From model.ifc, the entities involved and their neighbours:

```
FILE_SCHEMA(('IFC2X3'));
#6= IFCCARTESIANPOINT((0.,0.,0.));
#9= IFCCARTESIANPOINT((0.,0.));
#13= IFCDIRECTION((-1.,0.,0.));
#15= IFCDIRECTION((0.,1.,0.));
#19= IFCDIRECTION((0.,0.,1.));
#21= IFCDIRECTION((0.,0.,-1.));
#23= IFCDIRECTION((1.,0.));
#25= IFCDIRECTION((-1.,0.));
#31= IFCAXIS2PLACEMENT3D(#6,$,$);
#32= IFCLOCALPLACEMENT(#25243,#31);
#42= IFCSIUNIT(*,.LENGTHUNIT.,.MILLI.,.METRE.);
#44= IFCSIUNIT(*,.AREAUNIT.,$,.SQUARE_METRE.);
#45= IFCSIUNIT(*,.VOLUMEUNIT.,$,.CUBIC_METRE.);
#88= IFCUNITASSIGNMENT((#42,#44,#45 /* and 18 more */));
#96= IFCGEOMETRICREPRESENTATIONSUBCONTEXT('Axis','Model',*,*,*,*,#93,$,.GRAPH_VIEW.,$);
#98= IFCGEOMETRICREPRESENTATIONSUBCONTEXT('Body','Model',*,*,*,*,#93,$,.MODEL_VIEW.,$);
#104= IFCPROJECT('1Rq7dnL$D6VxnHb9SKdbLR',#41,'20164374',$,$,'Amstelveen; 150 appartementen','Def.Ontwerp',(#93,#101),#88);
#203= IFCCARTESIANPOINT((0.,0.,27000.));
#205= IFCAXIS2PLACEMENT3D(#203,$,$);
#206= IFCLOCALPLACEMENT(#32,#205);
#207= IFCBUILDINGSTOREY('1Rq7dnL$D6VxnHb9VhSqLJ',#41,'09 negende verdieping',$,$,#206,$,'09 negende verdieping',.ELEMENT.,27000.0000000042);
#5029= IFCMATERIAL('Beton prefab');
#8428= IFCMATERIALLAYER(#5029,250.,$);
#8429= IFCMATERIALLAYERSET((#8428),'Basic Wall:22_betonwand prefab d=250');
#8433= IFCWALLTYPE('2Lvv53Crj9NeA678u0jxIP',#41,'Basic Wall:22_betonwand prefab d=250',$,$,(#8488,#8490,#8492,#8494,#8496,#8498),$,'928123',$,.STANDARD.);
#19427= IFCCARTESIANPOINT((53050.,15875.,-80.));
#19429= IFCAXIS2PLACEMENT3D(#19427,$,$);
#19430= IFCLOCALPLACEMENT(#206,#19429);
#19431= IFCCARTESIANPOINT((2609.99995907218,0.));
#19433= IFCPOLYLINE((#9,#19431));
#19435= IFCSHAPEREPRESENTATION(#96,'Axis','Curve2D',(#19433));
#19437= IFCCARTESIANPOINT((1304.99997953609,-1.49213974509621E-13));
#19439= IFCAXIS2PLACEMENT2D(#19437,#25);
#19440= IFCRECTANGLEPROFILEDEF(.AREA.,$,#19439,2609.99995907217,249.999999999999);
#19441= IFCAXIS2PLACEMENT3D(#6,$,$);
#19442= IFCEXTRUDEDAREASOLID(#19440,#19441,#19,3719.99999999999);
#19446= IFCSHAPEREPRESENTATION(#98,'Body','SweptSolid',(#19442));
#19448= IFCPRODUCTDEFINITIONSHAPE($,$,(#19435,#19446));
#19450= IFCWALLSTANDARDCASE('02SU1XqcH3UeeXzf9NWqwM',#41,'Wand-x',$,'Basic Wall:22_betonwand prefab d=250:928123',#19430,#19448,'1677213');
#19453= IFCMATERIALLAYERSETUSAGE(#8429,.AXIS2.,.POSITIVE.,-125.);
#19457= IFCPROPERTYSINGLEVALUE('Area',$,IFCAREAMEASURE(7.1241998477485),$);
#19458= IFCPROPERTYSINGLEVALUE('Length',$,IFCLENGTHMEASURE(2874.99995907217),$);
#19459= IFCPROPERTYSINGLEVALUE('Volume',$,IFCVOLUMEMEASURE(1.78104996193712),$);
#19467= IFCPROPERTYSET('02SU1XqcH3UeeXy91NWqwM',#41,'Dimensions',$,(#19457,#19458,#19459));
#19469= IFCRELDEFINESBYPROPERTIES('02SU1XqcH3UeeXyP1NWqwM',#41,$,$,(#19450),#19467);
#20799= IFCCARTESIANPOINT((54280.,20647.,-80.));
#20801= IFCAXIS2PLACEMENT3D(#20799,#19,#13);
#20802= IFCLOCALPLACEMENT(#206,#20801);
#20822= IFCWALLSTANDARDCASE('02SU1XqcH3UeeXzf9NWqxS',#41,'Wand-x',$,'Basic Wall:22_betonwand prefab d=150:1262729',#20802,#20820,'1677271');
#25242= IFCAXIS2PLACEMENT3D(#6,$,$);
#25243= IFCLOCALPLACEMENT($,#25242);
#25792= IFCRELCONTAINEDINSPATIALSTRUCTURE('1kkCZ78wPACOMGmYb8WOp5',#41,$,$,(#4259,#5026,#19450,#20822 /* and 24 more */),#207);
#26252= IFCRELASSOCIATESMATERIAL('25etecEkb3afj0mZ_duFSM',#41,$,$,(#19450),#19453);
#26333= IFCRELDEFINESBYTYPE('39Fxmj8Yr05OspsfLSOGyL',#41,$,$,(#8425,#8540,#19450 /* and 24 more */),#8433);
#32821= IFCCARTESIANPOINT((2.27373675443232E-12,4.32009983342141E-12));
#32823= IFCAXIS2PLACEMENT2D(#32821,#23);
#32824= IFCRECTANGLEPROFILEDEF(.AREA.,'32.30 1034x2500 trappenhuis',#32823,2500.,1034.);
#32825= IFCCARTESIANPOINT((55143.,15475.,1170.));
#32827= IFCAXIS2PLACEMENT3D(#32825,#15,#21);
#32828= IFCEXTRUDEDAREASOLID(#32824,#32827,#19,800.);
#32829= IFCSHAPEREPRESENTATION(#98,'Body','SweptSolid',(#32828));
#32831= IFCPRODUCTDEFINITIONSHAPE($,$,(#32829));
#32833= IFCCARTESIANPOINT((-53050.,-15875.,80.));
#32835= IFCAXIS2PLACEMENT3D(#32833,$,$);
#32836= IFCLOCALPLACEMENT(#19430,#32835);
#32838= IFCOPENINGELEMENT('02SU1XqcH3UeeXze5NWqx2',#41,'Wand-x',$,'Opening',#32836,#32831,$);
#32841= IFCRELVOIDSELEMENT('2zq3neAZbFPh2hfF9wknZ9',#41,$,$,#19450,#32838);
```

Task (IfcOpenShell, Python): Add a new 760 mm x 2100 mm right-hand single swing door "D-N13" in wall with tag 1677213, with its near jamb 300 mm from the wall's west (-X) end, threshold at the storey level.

```python
import numpy as np
import ifcopenshell
import ifcopenshell.api.feature
import ifcopenshell.api.geometry
import ifcopenshell.api.pset
import ifcopenshell.api.root
import ifcopenshell.api.spatial
import ifcopenshell.api.type
import ifcopenshell.geom
import ifcopenshell.util.element
import ifcopenshell.util.placement
import ifcopenshell.util.representation
import ifcopenshell.util.shape
import ifcopenshell.util.unit

model = ifcopenshell.open("model.ifc")
unit_scale = ifcopenshell.util.unit.calculate_unit_scale(model)
area_scale = ifcopenshell.util.unit.calculate_unit_scale(model, "AREAUNIT")
volume_scale = ifcopenshell.util.unit.calculate_unit_scale(model, "VOLUMEUNIT")
settings = ifcopenshell.geom.settings()


def volume(element):
    """Net volume in cubic metres, openings subtracted."""
    shape = ifcopenshell.geom.create_shape(settings, element)
    return ifcopenshell.util.shape.get_volume(shape.geometry)


wall = model.by_guid("02SU1XqcH3UeeXzf9NWqwM")
storey = ifcopenshell.util.element.get_container(wall, ifc_class="IfcBuildingStorey")
context = ifcopenshell.util.representation.get_context(model, "Model", "Body", "MODEL_VIEW")
before = volume(wall)

width, height, from_end, sill = 0.76, 2.1, 0.3, 0.0  # metres

# The wall runs along its own X axis, and the end named is its -X end.
wall_shape = ifcopenshell.geom.create_shape(settings, wall)
x, y, z = ifcopenshell.util.shape.get_vertices(wall_shape.geometry).T
start = x.min() + from_end
face, thickness = float(y.min()), float(y.max() - y.min())
wall_matrix = ifcopenshell.util.placement.get_local_placement(wall.ObjectPlacement)
level = ifcopenshell.util.placement.get_local_placement(storey.ObjectPlacement)[2, 3]


def in_wall(x, y):
    """Placement at x, y metres in the wall's axes, at sill height."""
    matrix = wall_matrix.copy()
    matrix[:, 3] = wall_matrix @ np.array([x / unit_scale, y / unit_scale, 0.0, 1.0])
    matrix[2, 3] = level + sill / unit_scale
    return matrix


# Opening: a box that overshoots both wall faces by 50 mm.
opening = ifcopenshell.api.root.create_entity(model, ifc_class="IfcOpeningElement")
box = ifcopenshell.api.geometry.add_wall_representation(
    model, context=context, length=width, height=height, thickness=thickness + 0.1
)
ifcopenshell.api.geometry.assign_representation(model, product=opening, representation=box)
ifcopenshell.api.geometry.edit_object_placement(model, product=opening, matrix=in_wall(start, face - 0.05), is_si=False)
ifcopenshell.api.feature.add_feature(model, feature=opening, element=wall)

door = ifcopenshell.api.root.create_entity(model, ifc_class="IfcDoor", name="D-N13")
door.OverallWidth, door.OverallHeight = width / unit_scale, height / unit_scale
body = ifcopenshell.api.geometry.add_door_representation(
    model,
    context=context,
    overall_width=door.OverallWidth,
    overall_height=door.OverallHeight,
    operation_type="SINGLE_SWING_RIGHT",
    lining_properties={"LiningDepth": thickness / unit_scale, "ThresholdDepth": thickness / unit_scale},
)
ifcopenshell.api.geometry.assign_representation(model, product=door, representation=body)
ifcopenshell.api.spatial.assign_container(model, products=[door], relating_structure=storey)
fills = ifcopenshell.api.feature.add_filling(model, opening=opening, element=door)
fills.OwnerHistory = door.OwnerHistory  # required in IFC2X3

# IFC2X3 keeps the operation on the door style.
style = ifcopenshell.api.root.create_entity(model, ifc_class="IfcDoorStyle", name="D-N13")
style.OperationType, style.ConstructionType = "SINGLE_SWING_RIGHT", "NOTDEFINED"
style.ParameterTakesPrecedence = style.Sizeable = False
ifcopenshell.api.type.assign_type(model, related_objects=[door], relating_type=style)

# The lining spans the wall, so the door starts at the wall face.
ifcopenshell.api.geometry.edit_object_placement(model, product=door, matrix=in_wall(start, face), is_si=False)

after = volume(wall)

# Update the wall's stored quantities.
pset = model.by_id(ifcopenshell.util.element.get_pset(wall, "Dimensions", should_inherit=False)["id"])
ifcopenshell.api.pset.edit_pset(model, pset=pset, properties={
    "Area": model.create_entity("IfcAreaMeasure", after / thickness / area_scale),
    "Volume": model.create_entity("IfcVolumeMeasure", after / volume_scale),
})

print(f"wall volume {before:.3f} -> {after:.3f} m3")

model.write("model-out.ifc")
```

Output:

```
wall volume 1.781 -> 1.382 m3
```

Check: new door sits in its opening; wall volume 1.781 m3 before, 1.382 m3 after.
